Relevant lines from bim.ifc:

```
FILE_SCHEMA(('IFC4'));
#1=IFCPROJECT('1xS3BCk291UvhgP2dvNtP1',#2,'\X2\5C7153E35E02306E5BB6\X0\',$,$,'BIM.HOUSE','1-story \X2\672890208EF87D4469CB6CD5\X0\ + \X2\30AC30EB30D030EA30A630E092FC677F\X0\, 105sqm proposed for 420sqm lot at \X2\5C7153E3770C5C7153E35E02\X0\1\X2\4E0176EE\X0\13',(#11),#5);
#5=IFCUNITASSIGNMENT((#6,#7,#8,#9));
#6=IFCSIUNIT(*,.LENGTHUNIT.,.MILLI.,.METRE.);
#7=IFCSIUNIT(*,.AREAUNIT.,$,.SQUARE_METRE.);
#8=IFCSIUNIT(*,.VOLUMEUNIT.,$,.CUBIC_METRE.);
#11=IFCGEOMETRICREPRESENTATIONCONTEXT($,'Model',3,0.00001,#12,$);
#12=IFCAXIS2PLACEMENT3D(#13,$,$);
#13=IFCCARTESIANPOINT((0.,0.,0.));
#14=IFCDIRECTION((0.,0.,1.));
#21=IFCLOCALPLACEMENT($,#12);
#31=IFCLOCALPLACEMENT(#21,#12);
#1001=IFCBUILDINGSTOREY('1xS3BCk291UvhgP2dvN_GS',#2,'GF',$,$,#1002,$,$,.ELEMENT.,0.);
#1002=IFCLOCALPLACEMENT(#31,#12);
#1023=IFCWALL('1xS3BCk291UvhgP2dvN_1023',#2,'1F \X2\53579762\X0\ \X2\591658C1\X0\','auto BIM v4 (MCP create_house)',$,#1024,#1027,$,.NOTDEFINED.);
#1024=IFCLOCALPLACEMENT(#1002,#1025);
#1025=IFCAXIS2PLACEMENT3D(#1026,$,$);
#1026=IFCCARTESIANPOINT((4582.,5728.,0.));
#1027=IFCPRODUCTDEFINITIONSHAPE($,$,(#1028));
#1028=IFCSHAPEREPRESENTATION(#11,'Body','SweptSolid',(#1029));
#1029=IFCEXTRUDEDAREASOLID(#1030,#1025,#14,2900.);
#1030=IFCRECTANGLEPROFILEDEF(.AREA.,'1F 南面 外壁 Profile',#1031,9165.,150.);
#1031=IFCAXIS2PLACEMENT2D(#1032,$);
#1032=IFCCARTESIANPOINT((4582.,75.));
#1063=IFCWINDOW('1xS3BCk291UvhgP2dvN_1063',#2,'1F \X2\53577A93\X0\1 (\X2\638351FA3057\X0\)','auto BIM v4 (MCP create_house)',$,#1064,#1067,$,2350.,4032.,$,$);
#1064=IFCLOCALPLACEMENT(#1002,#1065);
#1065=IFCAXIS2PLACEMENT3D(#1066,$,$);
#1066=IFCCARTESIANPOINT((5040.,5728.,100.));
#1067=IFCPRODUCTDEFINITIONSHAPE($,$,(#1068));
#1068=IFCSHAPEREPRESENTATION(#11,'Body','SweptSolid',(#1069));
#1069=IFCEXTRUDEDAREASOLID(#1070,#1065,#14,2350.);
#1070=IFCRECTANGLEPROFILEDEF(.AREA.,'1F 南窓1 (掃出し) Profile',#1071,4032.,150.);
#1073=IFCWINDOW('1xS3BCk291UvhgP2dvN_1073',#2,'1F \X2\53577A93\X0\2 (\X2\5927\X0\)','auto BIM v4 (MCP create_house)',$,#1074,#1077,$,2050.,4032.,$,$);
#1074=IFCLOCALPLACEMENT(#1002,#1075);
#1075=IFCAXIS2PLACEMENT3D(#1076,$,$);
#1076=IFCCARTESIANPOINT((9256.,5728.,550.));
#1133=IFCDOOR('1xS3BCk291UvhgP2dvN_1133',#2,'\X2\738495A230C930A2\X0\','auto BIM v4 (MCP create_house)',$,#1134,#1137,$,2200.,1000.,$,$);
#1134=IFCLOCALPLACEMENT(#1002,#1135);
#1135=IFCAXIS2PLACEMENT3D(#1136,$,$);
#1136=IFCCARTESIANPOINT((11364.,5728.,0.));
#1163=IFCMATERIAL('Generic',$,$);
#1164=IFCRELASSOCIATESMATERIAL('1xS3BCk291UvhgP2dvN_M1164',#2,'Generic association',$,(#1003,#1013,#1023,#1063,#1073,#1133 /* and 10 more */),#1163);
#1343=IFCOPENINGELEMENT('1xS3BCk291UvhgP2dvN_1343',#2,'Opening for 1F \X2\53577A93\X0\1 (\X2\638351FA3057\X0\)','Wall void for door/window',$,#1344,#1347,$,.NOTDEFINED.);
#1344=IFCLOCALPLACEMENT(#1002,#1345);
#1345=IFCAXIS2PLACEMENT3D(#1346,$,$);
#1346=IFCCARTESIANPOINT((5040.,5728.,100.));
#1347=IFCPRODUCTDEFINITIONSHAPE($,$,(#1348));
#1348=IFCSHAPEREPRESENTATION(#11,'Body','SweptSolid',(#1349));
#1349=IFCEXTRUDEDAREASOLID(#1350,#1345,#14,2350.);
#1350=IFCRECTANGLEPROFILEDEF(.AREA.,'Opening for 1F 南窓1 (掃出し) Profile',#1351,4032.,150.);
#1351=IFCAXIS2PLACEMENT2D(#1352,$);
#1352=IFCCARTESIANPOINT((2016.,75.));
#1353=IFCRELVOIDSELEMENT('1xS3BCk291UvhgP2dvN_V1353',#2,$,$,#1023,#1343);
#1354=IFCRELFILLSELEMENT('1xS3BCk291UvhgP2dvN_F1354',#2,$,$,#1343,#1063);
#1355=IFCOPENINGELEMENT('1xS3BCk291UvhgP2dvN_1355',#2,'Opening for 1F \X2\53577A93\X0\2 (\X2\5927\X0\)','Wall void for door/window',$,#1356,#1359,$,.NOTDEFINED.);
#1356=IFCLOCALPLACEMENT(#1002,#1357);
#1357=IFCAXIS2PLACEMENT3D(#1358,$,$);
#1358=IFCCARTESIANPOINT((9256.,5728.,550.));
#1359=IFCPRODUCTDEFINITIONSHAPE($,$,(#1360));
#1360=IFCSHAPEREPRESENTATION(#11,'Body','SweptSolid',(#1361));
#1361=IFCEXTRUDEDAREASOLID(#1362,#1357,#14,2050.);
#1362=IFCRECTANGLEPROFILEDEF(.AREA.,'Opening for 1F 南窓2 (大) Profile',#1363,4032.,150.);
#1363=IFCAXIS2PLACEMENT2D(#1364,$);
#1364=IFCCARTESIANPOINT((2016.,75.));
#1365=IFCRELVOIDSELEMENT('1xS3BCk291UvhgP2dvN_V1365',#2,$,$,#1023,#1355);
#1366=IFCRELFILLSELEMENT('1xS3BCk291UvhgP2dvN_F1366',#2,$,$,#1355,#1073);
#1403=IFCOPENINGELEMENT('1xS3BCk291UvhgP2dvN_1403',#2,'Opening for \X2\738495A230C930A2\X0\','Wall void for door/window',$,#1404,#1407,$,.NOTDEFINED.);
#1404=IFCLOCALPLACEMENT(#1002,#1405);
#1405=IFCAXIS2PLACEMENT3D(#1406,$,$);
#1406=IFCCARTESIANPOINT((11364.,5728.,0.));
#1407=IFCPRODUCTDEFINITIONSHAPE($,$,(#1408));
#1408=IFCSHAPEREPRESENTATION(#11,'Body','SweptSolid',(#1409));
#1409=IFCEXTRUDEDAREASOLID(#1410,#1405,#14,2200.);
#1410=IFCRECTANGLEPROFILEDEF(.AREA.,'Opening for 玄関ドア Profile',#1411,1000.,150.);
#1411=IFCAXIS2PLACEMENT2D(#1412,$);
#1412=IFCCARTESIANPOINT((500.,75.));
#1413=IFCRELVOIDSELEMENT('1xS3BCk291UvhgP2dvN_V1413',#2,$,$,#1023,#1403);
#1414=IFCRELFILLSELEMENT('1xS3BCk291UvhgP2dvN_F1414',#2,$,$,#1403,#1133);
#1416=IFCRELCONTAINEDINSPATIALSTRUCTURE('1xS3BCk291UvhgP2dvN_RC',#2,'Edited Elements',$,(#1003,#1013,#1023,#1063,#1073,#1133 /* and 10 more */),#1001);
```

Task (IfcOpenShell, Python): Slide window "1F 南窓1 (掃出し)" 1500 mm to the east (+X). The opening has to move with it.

```python
import ifcopenshell
import ifcopenshell.api.geometry
import ifcopenshell.util.placement
import ifcopenshell.util.unit

model = ifcopenshell.open("bim.ifc")
unit_scale = ifcopenshell.util.unit.calculate_unit_scale(model)

window = model.by_guid("1xS3BCk291UvhgP2dvN_1063")
opening = window.FillsVoids[0].RelatingOpeningElement
wall = opening.VoidsElements[0].RelatingBuildingElement

wall_matrix = ifcopenshell.util.placement.get_local_placement(wall.ObjectPlacement)
shift = wall_matrix[:3, 0] * 1.5 / unit_scale
before = ifcopenshell.util.placement.get_local_placement(window.ObjectPlacement)[:3, 3].copy()

# The window is not placed relative to its opening, so move both.
for product in (opening, window):
    matrix = ifcopenshell.util.placement.get_local_placement(product.ObjectPlacement)
    matrix[:3, 3] += shift
    ifcopenshell.api.geometry.edit_object_placement(model, product=product, matrix=matrix, is_si=False)

after = ifcopenshell.util.placement.get_local_placement(window.ObjectPlacement)[:3, 3]
print("window moved by", (after - before).round(3) + 0.0)

model.write("bim_updated.ifc")
```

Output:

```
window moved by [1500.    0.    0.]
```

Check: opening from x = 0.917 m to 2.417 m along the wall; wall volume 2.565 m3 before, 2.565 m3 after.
